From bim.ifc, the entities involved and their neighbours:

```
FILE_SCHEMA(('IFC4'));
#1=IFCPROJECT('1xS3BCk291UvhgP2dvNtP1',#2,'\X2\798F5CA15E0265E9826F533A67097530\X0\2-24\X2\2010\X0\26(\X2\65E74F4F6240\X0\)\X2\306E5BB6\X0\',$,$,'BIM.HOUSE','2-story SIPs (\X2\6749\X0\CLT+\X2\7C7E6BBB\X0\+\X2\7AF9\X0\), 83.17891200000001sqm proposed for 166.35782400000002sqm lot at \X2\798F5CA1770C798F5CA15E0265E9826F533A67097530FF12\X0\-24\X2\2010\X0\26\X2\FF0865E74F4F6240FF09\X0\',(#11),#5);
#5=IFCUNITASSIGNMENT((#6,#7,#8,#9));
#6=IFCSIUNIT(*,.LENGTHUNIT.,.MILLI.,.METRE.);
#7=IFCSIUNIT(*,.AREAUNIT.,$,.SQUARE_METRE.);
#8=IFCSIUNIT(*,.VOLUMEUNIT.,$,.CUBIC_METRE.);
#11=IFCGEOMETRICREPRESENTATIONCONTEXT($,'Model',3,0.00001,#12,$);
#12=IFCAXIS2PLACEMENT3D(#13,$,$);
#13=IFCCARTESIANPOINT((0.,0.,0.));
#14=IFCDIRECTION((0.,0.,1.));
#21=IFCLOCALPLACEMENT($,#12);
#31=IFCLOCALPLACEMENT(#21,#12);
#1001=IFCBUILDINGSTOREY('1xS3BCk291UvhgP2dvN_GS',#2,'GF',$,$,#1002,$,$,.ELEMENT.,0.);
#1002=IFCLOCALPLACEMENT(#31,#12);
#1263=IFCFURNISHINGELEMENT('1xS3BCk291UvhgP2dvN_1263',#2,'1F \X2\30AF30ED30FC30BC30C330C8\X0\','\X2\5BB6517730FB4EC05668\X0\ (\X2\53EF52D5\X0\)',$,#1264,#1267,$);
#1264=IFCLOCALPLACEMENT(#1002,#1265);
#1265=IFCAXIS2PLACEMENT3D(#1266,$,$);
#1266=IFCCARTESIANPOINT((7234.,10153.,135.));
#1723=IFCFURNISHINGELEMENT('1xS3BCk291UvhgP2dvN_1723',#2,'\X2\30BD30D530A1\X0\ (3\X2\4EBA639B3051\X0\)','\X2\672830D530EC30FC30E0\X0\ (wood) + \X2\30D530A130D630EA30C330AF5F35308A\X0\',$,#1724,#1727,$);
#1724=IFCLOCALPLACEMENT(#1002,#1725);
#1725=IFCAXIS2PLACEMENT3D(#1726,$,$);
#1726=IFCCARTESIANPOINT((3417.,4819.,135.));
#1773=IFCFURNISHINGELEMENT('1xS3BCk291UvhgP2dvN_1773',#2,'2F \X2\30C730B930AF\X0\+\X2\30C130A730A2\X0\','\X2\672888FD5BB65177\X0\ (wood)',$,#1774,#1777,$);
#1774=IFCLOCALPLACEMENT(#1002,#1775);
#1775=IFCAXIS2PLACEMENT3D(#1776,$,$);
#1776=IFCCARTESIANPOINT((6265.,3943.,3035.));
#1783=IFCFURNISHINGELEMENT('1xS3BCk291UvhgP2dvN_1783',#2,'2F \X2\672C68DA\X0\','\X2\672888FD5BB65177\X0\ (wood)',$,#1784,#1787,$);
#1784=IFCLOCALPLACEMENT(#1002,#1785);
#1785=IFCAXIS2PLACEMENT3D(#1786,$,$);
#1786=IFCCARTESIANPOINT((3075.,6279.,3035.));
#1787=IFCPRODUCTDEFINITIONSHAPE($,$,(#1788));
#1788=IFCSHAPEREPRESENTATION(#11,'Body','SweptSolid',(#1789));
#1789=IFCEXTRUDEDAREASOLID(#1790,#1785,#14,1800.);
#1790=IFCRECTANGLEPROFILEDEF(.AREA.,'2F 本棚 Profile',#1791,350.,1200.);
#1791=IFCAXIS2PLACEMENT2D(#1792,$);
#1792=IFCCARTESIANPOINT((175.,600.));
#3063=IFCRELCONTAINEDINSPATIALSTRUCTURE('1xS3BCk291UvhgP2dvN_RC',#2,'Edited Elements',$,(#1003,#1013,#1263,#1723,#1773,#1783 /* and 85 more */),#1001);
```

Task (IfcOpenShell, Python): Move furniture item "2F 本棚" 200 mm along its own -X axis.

```python
import ifcopenshell
import ifcopenshell.api.geometry
import ifcopenshell.util.placement
import ifcopenshell.util.unit

model = ifcopenshell.open("bim.ifc")
unit_scale = ifcopenshell.util.unit.calculate_unit_scale(model)

item = model.by_id(1783)
matrix = ifcopenshell.util.placement.get_local_placement(item.ObjectPlacement)
matrix[:3, 3] -= matrix[:3, 0] * 0.2 / unit_scale
ifcopenshell.api.geometry.edit_object_placement(model, product=item, matrix=matrix, is_si=False)

print(ifcopenshell.util.placement.get_local_placement(item.ObjectPlacement).round(3) + 0.0)

model.write("bim_updated.ifc")
```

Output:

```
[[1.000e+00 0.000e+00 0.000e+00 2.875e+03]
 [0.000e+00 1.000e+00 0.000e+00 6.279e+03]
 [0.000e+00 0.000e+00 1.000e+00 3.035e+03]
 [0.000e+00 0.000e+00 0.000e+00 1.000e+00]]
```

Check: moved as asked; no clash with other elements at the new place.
